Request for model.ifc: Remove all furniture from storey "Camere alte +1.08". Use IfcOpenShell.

First a look at what the model holds.

```python
import ifcopenshell
import ifcopenshell.util.element

model = ifcopenshell.open("model.ifc")
print(model.schema)
storey = next(s for s in model.by_type("IfcBuildingStorey") if s.Name == "Camere alte +1.08")
furniture = [e for e in ifcopenshell.util.element.get_decomposition(storey) if e.is_a("IfcFurnishingElement")]
seen = {}
for e in furniture:
    element_type = ifcopenshell.util.element.get_type(e)
    name = element_type.Name if element_type not in (None, e) else None
    seen[name] = seen.get(name, 0) + 1
for name, count in sorted(seen.items(), key=str):
    print(count, "x", name)
```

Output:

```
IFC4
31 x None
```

```python
import ifcopenshell
import ifcopenshell.api.root
import ifcopenshell.util.element

model = ifcopenshell.open("model.ifc")

storey = next(s for s in model.by_type("IfcBuildingStorey") if s.Name == "Camere alte +1.08")
furniture = [e for e in ifcopenshell.util.element.get_decomposition(storey) if e.is_a("IfcFurnishingElement")]

for e in furniture:
    ifcopenshell.api.root.remove_product(model, product=e)
print(len(furniture), "removed")

model.write("model_v2.ifc")
```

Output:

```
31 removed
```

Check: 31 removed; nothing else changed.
